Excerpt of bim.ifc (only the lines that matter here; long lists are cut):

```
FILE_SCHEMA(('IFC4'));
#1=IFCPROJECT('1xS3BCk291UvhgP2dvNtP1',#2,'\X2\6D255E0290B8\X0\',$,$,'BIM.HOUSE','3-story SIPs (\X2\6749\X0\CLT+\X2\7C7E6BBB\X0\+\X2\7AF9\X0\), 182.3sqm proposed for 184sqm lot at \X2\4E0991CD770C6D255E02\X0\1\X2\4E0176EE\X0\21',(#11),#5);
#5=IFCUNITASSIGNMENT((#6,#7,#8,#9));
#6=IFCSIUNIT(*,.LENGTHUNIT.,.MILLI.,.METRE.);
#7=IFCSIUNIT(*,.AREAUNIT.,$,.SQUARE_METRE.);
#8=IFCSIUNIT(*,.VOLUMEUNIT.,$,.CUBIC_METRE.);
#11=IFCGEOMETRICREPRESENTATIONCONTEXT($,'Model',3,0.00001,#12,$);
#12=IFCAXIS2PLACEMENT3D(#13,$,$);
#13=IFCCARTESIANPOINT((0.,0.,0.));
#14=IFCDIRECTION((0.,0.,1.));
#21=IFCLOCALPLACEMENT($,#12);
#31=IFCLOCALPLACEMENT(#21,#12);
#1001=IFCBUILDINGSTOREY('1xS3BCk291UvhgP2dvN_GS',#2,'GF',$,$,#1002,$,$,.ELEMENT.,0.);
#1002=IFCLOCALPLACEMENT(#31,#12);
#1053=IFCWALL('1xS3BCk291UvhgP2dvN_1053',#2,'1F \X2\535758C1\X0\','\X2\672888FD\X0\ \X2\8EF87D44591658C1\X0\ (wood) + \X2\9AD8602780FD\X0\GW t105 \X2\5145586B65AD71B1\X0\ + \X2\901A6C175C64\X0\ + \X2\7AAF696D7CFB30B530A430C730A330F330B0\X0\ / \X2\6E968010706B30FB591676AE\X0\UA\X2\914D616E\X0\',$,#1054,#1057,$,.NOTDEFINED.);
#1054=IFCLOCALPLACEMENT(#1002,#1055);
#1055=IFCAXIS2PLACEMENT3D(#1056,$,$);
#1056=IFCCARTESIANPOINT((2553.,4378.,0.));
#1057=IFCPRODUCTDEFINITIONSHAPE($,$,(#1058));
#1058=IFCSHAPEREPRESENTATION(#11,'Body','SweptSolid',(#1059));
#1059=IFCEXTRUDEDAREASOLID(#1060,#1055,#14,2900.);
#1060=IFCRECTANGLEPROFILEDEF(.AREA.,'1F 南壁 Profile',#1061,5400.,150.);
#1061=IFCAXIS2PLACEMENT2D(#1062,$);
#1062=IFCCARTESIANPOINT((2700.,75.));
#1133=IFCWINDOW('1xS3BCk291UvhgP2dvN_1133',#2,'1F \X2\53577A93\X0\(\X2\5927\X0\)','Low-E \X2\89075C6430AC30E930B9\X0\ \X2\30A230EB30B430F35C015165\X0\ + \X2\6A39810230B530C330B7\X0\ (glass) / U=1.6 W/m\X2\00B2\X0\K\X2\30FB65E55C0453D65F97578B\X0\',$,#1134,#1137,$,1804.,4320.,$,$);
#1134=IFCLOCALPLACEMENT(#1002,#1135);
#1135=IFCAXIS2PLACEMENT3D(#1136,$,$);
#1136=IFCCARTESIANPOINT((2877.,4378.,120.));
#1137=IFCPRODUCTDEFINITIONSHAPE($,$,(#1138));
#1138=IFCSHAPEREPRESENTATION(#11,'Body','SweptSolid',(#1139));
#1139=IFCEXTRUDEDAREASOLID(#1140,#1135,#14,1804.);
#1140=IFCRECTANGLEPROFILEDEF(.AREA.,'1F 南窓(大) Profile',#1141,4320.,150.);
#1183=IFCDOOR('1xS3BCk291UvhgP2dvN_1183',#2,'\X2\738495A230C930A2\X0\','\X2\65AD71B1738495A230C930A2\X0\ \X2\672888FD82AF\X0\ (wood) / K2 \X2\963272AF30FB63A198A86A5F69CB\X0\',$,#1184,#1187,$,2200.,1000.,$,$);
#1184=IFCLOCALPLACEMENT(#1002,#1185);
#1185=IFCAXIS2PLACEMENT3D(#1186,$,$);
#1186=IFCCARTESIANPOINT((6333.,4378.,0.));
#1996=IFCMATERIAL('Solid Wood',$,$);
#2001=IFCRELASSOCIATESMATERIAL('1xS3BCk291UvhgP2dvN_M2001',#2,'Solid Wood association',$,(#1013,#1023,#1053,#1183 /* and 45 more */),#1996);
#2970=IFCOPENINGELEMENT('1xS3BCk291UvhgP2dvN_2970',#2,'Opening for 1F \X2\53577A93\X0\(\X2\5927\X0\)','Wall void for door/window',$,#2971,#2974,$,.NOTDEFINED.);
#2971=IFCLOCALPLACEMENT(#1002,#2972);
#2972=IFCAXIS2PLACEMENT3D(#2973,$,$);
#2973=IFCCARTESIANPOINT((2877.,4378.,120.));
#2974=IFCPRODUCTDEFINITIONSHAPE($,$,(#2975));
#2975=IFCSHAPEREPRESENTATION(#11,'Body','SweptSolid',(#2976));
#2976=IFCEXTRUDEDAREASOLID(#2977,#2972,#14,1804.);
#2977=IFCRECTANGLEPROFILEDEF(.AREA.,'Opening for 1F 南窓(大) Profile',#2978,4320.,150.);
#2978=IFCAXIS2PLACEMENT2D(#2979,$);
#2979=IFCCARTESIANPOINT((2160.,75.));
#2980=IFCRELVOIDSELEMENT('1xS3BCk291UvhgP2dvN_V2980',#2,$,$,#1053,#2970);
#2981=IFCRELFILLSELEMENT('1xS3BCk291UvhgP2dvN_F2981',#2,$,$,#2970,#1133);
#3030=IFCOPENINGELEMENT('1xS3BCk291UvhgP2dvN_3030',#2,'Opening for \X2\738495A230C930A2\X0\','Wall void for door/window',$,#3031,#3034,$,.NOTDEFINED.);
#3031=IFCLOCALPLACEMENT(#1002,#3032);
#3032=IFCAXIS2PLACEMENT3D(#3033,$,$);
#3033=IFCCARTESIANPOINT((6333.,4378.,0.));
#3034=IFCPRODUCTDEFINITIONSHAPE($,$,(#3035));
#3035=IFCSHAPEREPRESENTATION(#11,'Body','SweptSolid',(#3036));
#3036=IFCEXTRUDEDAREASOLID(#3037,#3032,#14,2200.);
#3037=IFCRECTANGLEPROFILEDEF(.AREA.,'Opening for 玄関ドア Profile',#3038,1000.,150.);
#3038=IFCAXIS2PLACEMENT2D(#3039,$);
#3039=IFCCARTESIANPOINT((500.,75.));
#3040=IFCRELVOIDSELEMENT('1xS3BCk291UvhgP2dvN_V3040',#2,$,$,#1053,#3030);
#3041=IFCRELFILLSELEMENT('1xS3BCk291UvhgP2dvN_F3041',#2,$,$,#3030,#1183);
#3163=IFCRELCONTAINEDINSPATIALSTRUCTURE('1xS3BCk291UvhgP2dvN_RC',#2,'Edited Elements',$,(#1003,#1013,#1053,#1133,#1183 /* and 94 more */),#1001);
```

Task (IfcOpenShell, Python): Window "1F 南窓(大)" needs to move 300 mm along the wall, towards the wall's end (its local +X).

```python
import ifcopenshell
import ifcopenshell.api.geometry
import ifcopenshell.util.placement

model = ifcopenshell.open("bim.ifc")

window = model.by_guid("1xS3BCk291UvhgP2dvN_1133")
opening = window.FillsVoids[0].RelatingOpeningElement
wall = opening.VoidsElements[0].RelatingBuildingElement

wall_matrix = ifcopenshell.util.placement.get_local_placement(wall.ObjectPlacement)
shift = wall_matrix[:3, 0] * 300.0
before = ifcopenshell.util.placement.get_local_placement(window.ObjectPlacement)[:3, 3].copy()

# The window is not placed relative to its opening, so move both.
for product in (opening, window):
    matrix = ifcopenshell.util.placement.get_local_placement(product.ObjectPlacement)
    matrix[:3, 3] += shift
    ifcopenshell.api.geometry.edit_object_placement(model, product=product, matrix=matrix, is_si=False)

after = ifcopenshell.util.placement.get_local_placement(window.ObjectPlacement)[:3, 3]
print("window moved by", (after - before).round(3) + 0.0)

model.write("bim_edited.ifc")
```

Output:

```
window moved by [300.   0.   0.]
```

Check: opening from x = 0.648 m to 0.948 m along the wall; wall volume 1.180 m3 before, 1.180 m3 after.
